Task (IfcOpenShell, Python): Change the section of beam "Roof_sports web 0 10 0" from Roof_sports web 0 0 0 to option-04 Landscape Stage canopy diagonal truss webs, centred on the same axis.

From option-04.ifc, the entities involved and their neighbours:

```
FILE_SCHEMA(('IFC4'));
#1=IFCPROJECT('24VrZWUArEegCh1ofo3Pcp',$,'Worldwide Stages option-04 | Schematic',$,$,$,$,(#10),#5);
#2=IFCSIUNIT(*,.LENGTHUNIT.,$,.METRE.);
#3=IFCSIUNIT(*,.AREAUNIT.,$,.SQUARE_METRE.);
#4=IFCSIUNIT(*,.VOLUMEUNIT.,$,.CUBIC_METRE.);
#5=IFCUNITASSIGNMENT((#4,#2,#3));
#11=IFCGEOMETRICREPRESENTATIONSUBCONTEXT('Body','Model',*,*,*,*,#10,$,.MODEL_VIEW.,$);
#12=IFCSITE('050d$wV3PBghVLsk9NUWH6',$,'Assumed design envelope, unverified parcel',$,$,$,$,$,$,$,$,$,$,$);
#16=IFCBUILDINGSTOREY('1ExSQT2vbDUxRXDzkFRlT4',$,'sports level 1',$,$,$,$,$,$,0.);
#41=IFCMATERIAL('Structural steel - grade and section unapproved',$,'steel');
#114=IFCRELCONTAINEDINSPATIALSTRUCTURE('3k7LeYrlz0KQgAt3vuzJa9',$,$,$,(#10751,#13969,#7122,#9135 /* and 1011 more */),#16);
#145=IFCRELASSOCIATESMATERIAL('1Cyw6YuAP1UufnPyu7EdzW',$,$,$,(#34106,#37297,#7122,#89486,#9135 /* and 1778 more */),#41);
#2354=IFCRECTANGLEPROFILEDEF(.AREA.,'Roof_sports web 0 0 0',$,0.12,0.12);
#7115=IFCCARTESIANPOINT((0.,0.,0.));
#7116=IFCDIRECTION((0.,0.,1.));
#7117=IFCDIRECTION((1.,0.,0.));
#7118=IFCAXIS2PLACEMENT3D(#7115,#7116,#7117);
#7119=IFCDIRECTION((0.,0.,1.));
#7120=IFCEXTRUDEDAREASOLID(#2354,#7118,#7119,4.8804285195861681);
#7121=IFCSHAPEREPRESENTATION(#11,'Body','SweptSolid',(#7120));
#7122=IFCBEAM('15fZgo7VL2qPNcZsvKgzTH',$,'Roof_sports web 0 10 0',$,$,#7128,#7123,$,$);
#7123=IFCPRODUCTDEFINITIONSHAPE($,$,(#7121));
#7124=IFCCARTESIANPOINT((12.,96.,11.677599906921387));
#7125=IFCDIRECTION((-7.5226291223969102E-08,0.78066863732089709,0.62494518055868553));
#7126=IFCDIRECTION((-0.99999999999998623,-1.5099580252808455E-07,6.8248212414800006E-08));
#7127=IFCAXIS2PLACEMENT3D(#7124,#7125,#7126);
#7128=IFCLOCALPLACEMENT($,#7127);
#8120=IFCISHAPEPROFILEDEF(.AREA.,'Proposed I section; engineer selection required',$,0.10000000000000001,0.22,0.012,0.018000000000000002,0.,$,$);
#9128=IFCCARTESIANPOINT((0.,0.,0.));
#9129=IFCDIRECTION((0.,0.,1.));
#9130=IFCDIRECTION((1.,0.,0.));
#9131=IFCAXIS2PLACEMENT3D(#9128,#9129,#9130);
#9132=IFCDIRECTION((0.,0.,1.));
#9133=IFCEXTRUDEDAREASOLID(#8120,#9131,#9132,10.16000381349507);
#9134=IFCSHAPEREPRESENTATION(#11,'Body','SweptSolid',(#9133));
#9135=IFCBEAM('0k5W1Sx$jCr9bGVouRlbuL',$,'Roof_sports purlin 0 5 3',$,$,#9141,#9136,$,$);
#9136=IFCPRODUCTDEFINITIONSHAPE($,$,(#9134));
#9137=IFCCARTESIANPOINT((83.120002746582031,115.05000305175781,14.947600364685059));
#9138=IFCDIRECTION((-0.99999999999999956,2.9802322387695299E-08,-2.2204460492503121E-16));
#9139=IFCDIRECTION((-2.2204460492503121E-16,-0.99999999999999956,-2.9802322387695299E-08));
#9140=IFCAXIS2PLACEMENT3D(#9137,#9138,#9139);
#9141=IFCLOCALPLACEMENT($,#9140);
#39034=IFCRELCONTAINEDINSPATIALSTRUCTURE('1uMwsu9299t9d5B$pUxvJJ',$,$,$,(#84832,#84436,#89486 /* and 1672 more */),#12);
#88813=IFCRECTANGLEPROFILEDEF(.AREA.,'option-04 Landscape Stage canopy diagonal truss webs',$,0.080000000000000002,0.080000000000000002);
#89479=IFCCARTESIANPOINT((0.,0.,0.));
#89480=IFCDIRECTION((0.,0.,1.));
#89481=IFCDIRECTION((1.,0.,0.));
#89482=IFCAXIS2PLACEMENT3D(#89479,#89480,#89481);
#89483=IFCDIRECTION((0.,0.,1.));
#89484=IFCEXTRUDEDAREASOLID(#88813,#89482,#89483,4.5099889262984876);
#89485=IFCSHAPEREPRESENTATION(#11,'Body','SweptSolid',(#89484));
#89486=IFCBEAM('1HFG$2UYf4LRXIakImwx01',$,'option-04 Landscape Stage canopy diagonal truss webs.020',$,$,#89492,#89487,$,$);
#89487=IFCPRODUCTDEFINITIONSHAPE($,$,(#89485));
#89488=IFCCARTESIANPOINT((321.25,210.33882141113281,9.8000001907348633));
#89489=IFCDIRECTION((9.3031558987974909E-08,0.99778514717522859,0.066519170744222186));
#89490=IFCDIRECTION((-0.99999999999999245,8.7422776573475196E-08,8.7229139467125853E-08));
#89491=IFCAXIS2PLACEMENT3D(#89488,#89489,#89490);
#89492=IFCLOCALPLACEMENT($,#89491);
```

```python
import ifcopenshell
import ifcopenshell.util.element
import ifcopenshell.util.representation

model = ifcopenshell.open("option-04.ifc")

member = model.by_id(7122)
source = next(p for p in model.by_type("IfcRectangleProfileDef") if p.ProfileName == "option-04 Landscape Stage canopy diagonal truss webs")

body = ifcopenshell.util.representation.get_representation(member, "Model", "Body")
solid = body.Items[0]
old_profile = solid.SweptArea

# Copy the section's sizes but keep this member's own profile position.
profile = ifcopenshell.util.element.copy(model, source)
profile.Position = old_profile.Position
solid.SweptArea = profile
if not model.get_total_inverses(old_profile):
    ifcopenshell.util.element.remove_deep2(model, old_profile)

print(solid.SweptArea)

model.write("option-04_rev.ifc")
```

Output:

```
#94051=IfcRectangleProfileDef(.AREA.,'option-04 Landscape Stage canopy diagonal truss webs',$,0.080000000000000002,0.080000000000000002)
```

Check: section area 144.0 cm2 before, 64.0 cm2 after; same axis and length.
